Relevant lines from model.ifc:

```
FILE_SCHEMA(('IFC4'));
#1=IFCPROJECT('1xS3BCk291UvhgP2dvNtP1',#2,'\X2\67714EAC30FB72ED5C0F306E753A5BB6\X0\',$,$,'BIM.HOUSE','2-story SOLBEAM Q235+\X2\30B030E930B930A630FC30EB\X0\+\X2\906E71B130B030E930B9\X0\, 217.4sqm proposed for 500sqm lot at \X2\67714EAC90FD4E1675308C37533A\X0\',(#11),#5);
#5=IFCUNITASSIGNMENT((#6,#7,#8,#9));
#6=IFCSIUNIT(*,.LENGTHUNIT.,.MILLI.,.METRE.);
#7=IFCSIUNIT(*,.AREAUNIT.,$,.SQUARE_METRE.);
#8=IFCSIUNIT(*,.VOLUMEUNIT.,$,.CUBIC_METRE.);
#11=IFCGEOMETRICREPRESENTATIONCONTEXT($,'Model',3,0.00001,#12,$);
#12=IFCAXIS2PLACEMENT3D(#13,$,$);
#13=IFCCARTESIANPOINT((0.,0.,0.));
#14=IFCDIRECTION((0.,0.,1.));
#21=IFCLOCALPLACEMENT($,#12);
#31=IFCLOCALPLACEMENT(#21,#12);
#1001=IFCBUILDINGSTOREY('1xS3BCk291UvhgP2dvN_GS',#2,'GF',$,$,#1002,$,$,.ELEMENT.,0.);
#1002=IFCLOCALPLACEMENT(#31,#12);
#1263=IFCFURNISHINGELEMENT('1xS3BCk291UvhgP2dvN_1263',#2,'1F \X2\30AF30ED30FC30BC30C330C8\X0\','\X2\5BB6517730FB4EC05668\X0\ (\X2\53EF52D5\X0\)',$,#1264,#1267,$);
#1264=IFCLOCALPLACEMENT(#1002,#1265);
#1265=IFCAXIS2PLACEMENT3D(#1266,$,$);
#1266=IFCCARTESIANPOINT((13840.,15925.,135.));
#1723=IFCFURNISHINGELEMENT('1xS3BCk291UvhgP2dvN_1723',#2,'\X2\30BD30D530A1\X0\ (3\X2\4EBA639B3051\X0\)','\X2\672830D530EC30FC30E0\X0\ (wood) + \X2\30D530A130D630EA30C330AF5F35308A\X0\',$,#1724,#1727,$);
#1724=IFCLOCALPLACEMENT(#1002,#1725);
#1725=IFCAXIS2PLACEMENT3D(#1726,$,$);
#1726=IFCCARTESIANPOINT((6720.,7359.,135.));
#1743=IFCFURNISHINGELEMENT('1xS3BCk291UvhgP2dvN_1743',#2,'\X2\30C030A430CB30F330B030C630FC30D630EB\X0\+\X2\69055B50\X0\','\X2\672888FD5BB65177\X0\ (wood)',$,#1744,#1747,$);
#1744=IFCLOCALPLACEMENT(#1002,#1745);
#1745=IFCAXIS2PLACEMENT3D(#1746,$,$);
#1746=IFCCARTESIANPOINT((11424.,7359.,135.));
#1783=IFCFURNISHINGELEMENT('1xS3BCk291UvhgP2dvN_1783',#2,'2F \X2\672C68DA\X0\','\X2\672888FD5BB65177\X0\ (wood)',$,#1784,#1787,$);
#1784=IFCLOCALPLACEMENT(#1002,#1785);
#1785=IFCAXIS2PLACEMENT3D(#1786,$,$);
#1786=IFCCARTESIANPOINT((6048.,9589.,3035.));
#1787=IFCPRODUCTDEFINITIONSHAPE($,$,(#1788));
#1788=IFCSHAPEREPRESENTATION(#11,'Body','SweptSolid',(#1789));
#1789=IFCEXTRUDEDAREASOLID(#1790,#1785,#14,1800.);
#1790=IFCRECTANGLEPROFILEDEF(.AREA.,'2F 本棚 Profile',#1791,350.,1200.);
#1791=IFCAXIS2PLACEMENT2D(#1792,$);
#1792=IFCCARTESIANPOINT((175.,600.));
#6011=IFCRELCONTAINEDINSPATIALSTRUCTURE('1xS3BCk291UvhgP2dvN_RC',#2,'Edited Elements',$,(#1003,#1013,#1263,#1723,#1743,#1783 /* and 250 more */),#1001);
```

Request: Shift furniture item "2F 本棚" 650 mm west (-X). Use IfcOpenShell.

```python
import ifcopenshell
import ifcopenshell.api.geometry
import ifcopenshell.util.placement
import ifcopenshell.util.unit

model = ifcopenshell.open("model.ifc")
unit_scale = ifcopenshell.util.unit.calculate_unit_scale(model)

item = model.by_guid("1xS3BCk291UvhgP2dvN_1783")
matrix = ifcopenshell.util.placement.get_local_placement(item.ObjectPlacement)
matrix[0, 3] -= 0.65 / unit_scale
ifcopenshell.api.geometry.edit_object_placement(model, product=item, matrix=matrix, is_si=False)

print(ifcopenshell.util.placement.get_local_placement(item.ObjectPlacement).round(3) + 0.0)

model.write("model_updated.ifc")
```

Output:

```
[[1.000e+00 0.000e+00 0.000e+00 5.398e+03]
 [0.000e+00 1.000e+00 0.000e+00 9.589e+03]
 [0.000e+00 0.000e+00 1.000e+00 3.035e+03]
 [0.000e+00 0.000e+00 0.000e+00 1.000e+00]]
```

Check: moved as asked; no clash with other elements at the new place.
